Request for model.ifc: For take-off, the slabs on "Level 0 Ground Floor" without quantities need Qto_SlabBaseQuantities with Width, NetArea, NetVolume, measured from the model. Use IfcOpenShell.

First a look at what the model holds.

```python
import ifcopenshell
import ifcopenshell.util.element
import ifcopenshell.util.unit

model = ifcopenshell.open("model.ifc")
print(model.schema)
for unit_type in ("LENGTHUNIT", "AREAUNIT", "VOLUMEUNIT"):
    print(unit_type, ifcopenshell.util.unit.calculate_unit_scale(model, unit_type))
storey = next(s for s in model.by_type("IfcBuildingStorey") if s.Name == "Level 0 Ground Floor")
slabs = [e for e in ifcopenshell.util.element.get_decomposition(storey) if e.is_a("IfcSlab")]
for e in sorted(slabs, key=lambda e: e.id()):
    print(e.id(), e.is_a(), e.Name, list(ifcopenshell.util.element.get_psets(e, qtos_only=True)), sep=" | ")
```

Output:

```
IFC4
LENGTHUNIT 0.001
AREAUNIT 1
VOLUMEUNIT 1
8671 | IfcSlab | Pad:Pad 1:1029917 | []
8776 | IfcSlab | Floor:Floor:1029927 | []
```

```python
import ifcopenshell
import ifcopenshell.api.pset
import ifcopenshell.geom
import ifcopenshell.util.element
import ifcopenshell.util.shape
import ifcopenshell.util.unit

model = ifcopenshell.open("model.ifc")
unit_scale = ifcopenshell.util.unit.calculate_unit_scale(model)
area_scale = ifcopenshell.util.unit.calculate_unit_scale(model, "AREAUNIT")
volume_scale = ifcopenshell.util.unit.calculate_unit_scale(model, "VOLUMEUNIT")
settings = ifcopenshell.geom.settings()

storey = next(s for s in model.by_type("IfcBuildingStorey") if s.Name == "Level 0 Ground Floor")
slabs = [e for e in ifcopenshell.util.element.get_decomposition(storey) if e.is_a("IfcSlab")]

for e in sorted(slabs, key=lambda e: e.id()):
    if ifcopenshell.util.element.get_psets(e, qtos_only=True, should_inherit=False):
        continue
    # Geometry comes back in metres, in the element's own axes.
    shape = ifcopenshell.geom.create_shape(settings, e)
    values = {
        "Width": ifcopenshell.util.shape.get_z(shape.geometry) / unit_scale,
        "NetArea": ifcopenshell.util.shape.get_footprint_area(shape.geometry) / area_scale,
        "NetVolume": ifcopenshell.util.shape.get_volume(shape.geometry) / volume_scale,
    }
    qto = ifcopenshell.api.pset.add_qto(model, product=e, name="Qto_SlabBaseQuantities")
    ifcopenshell.api.pset.edit_qto(model, qto=qto, properties=values)
    print(e.id(), {k: round(v, 3) for k, v in values.items()})

model.write("model-out.ifc")
```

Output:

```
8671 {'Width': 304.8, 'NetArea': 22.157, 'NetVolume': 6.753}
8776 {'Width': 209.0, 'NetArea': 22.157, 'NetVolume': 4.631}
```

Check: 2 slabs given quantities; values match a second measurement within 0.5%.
